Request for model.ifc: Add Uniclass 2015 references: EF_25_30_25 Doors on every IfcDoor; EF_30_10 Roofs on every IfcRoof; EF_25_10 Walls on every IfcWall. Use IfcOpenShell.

First a look at what the model holds.

```python
import ifcopenshell

model = ifcopenshell.open("model.ifc")
print(model.schema)
print("classifications:", [c.Name for c in model.by_type("IfcClassification")])
for ifc_class in ("IfcDoor", "IfcRoof", "IfcStair", "IfcWall", "IfcWindow"):
    print(ifc_class, len(model.by_type(ifc_class)))
```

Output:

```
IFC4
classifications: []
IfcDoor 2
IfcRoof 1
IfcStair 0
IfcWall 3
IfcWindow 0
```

```python
import ifcopenshell
import ifcopenshell.api.classification

model = ifcopenshell.open("model.ifc")

system = ifcopenshell.api.classification.add_classification(model, classification="Uniclass 2015")

codes = {
    "IfcDoor": ("EF_25_30_25", "Doors"),
    "IfcRoof": ("EF_30_10", "Roofs"),
    "IfcWall": ("EF_25_10", "Walls"),
}
for ifc_class, (code, name) in codes.items():
    products = model.by_type(ifc_class)
    ifcopenshell.api.classification.add_reference(
        model, products=products, classification=system, identification=code, name=name
    )
    print(code, len(products))

model.write("model_updated.ifc")
```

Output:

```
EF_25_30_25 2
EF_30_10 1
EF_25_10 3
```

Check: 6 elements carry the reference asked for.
